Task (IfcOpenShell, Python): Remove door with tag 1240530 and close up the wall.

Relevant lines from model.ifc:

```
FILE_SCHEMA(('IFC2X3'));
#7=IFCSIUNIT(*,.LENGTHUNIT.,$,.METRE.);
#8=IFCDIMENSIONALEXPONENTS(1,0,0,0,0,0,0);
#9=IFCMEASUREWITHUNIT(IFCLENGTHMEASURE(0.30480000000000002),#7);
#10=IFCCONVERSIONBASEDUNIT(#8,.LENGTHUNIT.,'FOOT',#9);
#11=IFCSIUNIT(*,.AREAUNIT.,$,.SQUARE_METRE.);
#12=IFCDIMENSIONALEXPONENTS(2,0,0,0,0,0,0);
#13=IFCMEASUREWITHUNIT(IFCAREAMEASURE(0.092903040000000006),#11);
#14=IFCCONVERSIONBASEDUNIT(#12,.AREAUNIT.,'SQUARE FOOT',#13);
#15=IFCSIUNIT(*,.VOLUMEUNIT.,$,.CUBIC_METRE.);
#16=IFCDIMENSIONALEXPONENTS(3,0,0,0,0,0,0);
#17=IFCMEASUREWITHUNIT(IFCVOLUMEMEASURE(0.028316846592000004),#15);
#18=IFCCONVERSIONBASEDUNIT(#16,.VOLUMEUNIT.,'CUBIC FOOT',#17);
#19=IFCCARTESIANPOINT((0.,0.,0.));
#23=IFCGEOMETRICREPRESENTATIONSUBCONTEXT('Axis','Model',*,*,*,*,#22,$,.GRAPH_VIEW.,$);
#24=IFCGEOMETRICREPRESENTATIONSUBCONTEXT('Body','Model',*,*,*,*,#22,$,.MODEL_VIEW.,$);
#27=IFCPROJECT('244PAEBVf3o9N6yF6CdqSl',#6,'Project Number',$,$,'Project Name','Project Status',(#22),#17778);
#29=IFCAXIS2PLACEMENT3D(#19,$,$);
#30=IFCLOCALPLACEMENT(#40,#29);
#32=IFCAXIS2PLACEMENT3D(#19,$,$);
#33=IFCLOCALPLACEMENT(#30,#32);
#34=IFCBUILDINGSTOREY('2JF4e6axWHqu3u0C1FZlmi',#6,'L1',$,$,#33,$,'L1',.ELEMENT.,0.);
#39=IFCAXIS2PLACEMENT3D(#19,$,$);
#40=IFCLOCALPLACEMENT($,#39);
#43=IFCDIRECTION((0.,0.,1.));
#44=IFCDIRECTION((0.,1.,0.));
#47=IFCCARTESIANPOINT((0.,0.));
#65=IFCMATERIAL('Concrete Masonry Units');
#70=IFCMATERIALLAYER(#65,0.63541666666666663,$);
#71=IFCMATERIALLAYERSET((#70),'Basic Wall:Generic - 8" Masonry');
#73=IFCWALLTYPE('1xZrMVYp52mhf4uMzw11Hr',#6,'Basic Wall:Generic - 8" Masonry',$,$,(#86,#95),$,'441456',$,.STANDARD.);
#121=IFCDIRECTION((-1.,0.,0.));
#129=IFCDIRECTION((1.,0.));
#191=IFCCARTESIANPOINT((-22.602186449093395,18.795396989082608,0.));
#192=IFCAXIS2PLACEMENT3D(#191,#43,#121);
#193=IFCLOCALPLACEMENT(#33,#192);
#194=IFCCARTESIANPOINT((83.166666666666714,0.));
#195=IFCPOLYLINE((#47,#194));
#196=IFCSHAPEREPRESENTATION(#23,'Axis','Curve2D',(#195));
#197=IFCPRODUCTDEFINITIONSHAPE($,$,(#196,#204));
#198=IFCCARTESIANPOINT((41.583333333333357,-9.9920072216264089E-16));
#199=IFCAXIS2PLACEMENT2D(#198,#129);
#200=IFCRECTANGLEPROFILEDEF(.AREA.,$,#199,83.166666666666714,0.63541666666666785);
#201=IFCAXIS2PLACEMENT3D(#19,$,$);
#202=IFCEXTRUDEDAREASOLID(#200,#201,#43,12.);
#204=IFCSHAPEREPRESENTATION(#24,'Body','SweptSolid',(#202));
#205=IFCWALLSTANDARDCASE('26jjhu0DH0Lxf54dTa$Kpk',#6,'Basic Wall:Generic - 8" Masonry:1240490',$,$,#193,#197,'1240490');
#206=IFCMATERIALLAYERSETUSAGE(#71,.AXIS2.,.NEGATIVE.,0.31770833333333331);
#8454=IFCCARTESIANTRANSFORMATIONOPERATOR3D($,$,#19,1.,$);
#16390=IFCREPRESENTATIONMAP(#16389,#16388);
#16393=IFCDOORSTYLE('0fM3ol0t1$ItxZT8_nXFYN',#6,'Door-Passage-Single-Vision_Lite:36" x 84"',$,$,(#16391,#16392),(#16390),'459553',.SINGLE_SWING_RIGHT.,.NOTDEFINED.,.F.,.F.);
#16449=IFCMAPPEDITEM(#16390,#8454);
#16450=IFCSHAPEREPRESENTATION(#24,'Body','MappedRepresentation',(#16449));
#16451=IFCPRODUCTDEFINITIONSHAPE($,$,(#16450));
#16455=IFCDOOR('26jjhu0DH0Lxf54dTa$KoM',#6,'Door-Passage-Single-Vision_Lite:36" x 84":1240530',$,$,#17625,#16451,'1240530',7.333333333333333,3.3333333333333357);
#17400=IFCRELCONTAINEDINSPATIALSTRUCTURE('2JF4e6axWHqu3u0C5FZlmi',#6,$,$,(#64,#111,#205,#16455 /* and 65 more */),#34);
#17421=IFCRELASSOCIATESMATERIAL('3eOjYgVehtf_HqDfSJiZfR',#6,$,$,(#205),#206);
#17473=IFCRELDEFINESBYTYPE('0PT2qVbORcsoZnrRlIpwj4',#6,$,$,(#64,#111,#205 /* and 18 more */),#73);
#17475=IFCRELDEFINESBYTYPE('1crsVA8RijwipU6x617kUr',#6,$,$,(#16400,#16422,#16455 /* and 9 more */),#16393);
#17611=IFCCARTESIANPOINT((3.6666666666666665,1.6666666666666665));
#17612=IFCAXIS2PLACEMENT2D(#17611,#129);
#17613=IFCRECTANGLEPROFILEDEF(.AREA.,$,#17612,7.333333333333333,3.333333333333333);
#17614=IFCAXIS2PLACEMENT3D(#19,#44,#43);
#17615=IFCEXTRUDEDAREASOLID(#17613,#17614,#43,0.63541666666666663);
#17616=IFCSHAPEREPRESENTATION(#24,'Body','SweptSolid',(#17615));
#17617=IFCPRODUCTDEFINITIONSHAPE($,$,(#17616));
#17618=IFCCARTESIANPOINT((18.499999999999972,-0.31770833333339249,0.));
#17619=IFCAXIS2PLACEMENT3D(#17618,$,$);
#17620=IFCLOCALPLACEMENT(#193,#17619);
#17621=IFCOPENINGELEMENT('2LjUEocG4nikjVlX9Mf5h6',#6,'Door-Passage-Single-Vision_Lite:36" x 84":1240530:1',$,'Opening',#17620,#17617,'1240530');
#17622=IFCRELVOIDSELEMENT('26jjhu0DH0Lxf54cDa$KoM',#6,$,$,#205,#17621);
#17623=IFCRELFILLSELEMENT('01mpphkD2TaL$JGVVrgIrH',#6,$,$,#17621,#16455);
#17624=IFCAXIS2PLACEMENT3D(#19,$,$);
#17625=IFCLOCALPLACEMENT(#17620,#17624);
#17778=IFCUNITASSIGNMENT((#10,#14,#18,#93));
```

```python
import ifcopenshell
import ifcopenshell.api.feature
import ifcopenshell.api.root
import ifcopenshell.geom
import ifcopenshell.util.shape

model = ifcopenshell.open("model.ifc")
settings = ifcopenshell.geom.settings()


def volume(element):
    """Net volume in cubic metres, openings subtracted."""
    shape = ifcopenshell.geom.create_shape(settings, element)
    return ifcopenshell.util.shape.get_volume(shape.geometry)


door = model.by_guid("26jjhu0DH0Lxf54dTa$KoM")
opening = door.FillsVoids[0].RelatingOpeningElement
wall = opening.VoidsElements[0].RelatingBuildingElement
before = volume(wall)

ifcopenshell.api.root.remove_product(model, product=door)
ifcopenshell.api.feature.remove_feature(model, feature=opening)

after = volume(wall)

print(f"wall volume {before:.3f} -> {after:.3f} m3")

model.write("model-out.ifc")
```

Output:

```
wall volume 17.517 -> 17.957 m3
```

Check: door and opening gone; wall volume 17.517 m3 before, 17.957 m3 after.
